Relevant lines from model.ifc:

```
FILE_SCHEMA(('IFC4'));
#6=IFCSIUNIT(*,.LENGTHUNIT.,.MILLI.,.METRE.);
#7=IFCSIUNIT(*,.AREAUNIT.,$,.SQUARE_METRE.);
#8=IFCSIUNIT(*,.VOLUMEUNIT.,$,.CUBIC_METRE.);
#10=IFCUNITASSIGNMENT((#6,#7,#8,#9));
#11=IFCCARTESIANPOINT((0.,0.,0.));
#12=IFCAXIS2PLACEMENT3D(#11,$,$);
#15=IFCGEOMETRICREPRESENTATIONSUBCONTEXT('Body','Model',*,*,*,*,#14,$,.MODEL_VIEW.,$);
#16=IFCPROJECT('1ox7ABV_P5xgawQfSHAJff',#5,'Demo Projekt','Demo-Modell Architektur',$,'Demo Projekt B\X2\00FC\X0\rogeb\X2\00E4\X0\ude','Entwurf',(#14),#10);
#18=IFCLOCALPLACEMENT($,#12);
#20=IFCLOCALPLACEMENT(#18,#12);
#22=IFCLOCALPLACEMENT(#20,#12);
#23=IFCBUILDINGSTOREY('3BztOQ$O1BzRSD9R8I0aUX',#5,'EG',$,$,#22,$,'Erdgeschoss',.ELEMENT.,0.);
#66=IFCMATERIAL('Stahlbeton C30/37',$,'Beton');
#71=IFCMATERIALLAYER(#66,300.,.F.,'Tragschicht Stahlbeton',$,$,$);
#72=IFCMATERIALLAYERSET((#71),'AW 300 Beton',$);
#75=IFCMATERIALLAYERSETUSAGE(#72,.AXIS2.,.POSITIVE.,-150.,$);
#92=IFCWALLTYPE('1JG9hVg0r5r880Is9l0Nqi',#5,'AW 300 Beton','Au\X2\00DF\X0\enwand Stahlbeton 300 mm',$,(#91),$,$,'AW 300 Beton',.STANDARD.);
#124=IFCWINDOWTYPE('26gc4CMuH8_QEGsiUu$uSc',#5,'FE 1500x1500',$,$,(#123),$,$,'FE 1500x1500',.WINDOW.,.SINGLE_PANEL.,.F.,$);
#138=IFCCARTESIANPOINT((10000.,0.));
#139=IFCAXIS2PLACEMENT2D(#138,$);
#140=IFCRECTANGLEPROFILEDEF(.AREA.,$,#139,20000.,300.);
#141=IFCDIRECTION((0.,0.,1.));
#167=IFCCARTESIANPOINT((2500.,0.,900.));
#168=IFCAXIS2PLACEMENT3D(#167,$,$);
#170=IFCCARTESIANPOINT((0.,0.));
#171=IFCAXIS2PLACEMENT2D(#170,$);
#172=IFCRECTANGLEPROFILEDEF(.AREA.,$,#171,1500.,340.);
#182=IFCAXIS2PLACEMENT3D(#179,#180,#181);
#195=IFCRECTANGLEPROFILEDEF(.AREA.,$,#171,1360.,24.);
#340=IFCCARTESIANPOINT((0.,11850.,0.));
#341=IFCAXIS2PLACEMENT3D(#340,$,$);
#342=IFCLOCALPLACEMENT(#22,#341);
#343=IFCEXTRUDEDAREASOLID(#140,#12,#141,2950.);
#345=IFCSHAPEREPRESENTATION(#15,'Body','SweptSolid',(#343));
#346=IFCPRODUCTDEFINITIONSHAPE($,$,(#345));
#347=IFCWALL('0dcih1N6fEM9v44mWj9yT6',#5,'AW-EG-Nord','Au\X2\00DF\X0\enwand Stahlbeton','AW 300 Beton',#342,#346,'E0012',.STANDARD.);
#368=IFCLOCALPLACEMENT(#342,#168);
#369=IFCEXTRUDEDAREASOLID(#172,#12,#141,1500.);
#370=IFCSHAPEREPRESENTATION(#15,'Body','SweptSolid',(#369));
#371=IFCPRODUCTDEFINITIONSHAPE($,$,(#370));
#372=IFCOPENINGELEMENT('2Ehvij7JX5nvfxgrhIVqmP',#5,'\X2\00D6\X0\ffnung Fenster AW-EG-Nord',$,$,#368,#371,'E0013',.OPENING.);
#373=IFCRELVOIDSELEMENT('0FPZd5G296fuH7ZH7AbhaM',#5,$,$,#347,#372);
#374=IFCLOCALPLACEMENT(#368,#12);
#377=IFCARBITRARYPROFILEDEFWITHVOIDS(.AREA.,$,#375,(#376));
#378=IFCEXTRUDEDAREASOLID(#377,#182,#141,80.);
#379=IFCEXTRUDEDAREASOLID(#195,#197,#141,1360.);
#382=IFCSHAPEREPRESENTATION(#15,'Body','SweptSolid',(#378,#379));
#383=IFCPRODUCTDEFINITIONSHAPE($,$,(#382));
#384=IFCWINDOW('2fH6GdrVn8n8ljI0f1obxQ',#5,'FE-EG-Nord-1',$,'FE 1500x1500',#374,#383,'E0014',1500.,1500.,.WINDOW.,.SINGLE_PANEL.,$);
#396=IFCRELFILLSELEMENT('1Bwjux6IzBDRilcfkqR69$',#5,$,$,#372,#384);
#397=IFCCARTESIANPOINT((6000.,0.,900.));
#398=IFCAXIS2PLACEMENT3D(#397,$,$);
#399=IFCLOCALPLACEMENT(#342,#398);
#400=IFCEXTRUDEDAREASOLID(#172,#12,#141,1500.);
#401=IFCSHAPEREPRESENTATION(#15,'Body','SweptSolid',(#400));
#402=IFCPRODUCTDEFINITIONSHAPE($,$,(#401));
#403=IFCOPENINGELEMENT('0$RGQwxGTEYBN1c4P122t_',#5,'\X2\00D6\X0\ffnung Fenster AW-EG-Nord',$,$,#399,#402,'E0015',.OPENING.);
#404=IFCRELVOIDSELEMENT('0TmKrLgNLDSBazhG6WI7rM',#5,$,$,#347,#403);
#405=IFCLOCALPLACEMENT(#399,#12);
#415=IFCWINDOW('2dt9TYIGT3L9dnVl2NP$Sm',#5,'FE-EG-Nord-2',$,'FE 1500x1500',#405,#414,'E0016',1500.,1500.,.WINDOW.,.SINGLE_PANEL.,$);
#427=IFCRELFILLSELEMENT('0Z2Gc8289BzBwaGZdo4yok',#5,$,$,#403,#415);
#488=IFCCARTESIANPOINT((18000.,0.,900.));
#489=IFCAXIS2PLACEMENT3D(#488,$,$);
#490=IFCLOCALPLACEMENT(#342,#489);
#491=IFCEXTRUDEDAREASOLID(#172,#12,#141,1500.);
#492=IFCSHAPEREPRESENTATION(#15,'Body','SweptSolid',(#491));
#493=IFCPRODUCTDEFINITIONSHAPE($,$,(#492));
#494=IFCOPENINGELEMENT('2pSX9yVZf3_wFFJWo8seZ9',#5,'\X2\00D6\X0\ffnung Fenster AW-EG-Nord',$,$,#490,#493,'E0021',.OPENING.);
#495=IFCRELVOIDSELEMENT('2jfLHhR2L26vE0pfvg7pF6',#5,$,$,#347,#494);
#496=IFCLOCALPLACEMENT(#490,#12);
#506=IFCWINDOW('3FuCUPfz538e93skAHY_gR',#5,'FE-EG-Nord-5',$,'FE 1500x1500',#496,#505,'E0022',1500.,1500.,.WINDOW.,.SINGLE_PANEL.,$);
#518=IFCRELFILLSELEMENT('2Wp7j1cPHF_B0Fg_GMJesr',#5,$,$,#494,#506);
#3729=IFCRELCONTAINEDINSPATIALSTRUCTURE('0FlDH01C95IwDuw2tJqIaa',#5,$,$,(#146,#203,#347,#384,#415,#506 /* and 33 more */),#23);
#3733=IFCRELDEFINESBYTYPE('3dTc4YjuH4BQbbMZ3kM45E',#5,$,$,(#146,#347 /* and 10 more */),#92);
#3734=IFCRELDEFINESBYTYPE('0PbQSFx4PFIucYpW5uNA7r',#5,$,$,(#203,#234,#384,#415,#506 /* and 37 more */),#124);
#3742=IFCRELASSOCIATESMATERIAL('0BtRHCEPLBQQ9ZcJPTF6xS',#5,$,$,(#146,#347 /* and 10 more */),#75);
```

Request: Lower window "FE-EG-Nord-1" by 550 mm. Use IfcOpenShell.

```python
import numpy as np
import ifcopenshell
import ifcopenshell.api.geometry
import ifcopenshell.util.placement
import ifcopenshell.util.unit

model = ifcopenshell.open("model.ifc")
unit_scale = ifcopenshell.util.unit.calculate_unit_scale(model)

window = model.by_id(384)
opening = window.FillsVoids[0].RelatingOpeningElement
dz = -0.55 / unit_scale

shift = np.array([0.0, 0.0, dz])
# The window is placed relative to its opening, so it follows when the opening moves.
matrix = ifcopenshell.util.placement.get_local_placement(opening.ObjectPlacement)
matrix[:3, 3] += shift
ifcopenshell.api.geometry.edit_object_placement(
    model, product=opening, matrix=matrix, is_si=False, should_transform_children=True
)

print(f"moved by {dz * unit_scale:+.3f} m")

model.write("model_edited.ifc")
```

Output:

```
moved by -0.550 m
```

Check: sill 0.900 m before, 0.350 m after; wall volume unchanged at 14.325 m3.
